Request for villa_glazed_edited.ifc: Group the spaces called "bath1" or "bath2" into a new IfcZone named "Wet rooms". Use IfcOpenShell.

First a look at what the model holds.

```python
import ifcopenshell

model = ifcopenshell.open("villa_glazed_edited.ifc")
print(model.schema)
seen = {}
for space in model.by_type("IfcSpace"):
    seen[space.LongName] = seen.get(space.LongName, 0) + 1
for name, count in sorted(seen.items(), key=str):
    print(count, "x", name)
print("zones:", [z.Name for z in model.by_type("IfcZone")][:20])
```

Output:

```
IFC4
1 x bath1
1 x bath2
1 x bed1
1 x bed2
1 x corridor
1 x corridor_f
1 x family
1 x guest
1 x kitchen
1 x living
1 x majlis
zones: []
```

```python
import ifcopenshell
import ifcopenshell.api.group
import ifcopenshell.api.root

model = ifcopenshell.open("villa_glazed_edited.ifc")

names = {"bath1", "bath2"}
spaces = [s for s in model.by_type("IfcSpace") if s.LongName in names]

zone = ifcopenshell.api.root.create_entity(model, ifc_class="IfcZone", name="Wet rooms")
ifcopenshell.api.group.assign_group(model, products=spaces, group=zone)
print(len(spaces), "spaces in", zone.Name)

model.write("villa_glazed_edited_updated.ifc")
```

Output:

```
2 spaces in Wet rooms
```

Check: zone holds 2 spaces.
